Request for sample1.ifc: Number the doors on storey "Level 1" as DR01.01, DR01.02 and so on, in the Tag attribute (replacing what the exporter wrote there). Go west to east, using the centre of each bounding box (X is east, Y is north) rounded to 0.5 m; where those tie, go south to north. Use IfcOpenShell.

First a look at what the model holds.

```python
import ifcopenshell
import ifcopenshell.util.element
import ifcopenshell.util.placement

model = ifcopenshell.open("sample1.ifc")
print(model.schema)
storey = next(s for s in model.by_type("IfcBuildingStorey") if s.Name == "Level 1")
doors = [e for e in ifcopenshell.util.element.get_decomposition(storey) if e.is_a("IfcDoor")]
for e in sorted(doors, key=lambda e: e.id()):
    origin = ifcopenshell.util.placement.get_local_placement(e.ObjectPlacement)[:3, 3]
    print(e.id(), e.Tag, e.Name, origin.round(2) + 0.0, sep=" | ")
```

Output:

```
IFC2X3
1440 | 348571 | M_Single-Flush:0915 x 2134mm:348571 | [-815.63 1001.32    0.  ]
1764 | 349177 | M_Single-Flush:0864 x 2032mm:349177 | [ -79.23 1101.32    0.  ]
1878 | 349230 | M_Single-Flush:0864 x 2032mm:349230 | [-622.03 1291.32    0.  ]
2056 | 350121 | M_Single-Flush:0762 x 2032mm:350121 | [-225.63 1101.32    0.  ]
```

```python
import ifcopenshell
import ifcopenshell.geom
import ifcopenshell.util.element
import ifcopenshell.util.shape

model = ifcopenshell.open("sample1.ifc")
settings = ifcopenshell.geom.settings()
settings.set("use-world-coords", True)


def centre(element):
    shape = ifcopenshell.geom.create_shape(settings, element)
    return ifcopenshell.util.shape.get_bbox_centroid(shape.geometry)


storey = next(s for s in model.by_type("IfcBuildingStorey") if s.Name == "Level 1")
doors = [e for e in ifcopenshell.util.element.get_decomposition(storey) if e.is_a("IfcDoor")]

# Insertion points can sit at a corner or the storey origin, so sort by the geometry (in metres).
centres = {e: centre(e) for e in doors}
doors.sort(key=lambda e: (round(centres[e][0] / 0.5), centres[e][1]))

for i, e in enumerate(doors, start=1):
    number = f"DR01.{i:02d}"
    e.Tag = number
    print(e.id(), number)

model.write("sample1_updated.ifc")
```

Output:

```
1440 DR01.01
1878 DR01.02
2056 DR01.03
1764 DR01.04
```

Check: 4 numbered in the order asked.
